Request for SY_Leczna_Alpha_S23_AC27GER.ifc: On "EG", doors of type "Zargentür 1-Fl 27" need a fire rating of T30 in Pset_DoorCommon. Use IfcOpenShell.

First a look at what the model holds.

```python
import ifcopenshell
import ifcopenshell.util.element

model = ifcopenshell.open("SY_Leczna_Alpha_S23_AC27GER.ifc")
print(model.schema)
storey = next(s for s in model.by_type("IfcBuildingStorey") if s.Name == "EG")
doors = [e for e in ifcopenshell.util.element.get_decomposition(storey) if e.is_a("IfcDoor")]
seen = {}
for e in doors:
    element_type = ifcopenshell.util.element.get_type(e)
    key = (element_type.Name if element_type != e and element_type else None, ifcopenshell.util.element.get_pset(e, "Pset_DoorCommon", "FireRating"))
    seen[key] = seen.get(key, 0) + 1
for (name, value), count in sorted(seen.items(), key=str):
    print(count, "x", name, "|", value)
```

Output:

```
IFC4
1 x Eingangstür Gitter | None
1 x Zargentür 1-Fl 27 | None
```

```python
import ifcopenshell
import ifcopenshell.api.pset
import ifcopenshell.util.element

model = ifcopenshell.open("SY_Leczna_Alpha_S23_AC27GER.ifc")

storey = next(s for s in model.by_type("IfcBuildingStorey") if s.Name == "EG")
doors = [e for e in ifcopenshell.util.element.get_decomposition(storey) if e.is_a("IfcDoor")]

count = 0
for e in doors:
    element_type = ifcopenshell.util.element.get_type(e)
    if element_type in (None, e) or element_type.Name != "Zargentür 1-Fl 27":
        continue
    # add_pset returns the element's existing set when there is one.
    pset = ifcopenshell.api.pset.add_pset(model, product=e, name="Pset_DoorCommon")
    ifcopenshell.api.pset.edit_pset(model, pset=pset, properties={"FireRating": "T30"})
    count += 1

print(count, "doors updated")

model.write("SY_Leczna_Alpha_S23_AC27GER-out.ifc")
```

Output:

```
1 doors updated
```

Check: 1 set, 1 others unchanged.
